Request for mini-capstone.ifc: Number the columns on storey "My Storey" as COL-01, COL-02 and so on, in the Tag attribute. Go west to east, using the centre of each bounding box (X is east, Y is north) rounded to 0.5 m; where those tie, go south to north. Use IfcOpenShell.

First a look at what the model holds.

```python
import ifcopenshell
import ifcopenshell.util.element
import ifcopenshell.util.placement

model = ifcopenshell.open("mini-capstone.ifc")
print(model.schema)
storey = next(s for s in model.by_type("IfcBuildingStorey") if s.Name == "My Storey")
columns = [e for e in ifcopenshell.util.element.get_decomposition(storey) if e.is_a("IfcColumn")]
for e in sorted(columns, key=lambda e: e.id()):
    origin = ifcopenshell.util.placement.get_local_placement(e.ObjectPlacement)[:3, 3]
    print(e.id(), e.Tag, e.Name, origin.round(2) + 0.0, sep=" | ")
```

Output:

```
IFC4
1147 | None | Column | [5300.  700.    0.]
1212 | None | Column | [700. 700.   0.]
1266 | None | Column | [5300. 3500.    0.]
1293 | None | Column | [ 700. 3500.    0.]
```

```python
import ifcopenshell
import ifcopenshell.geom
import ifcopenshell.util.element
import ifcopenshell.util.shape

model = ifcopenshell.open("mini-capstone.ifc")
settings = ifcopenshell.geom.settings()
settings.set("use-world-coords", True)


def centre(element):
    shape = ifcopenshell.geom.create_shape(settings, element)
    return ifcopenshell.util.shape.get_bbox_centroid(shape.geometry)


storey = next(s for s in model.by_type("IfcBuildingStorey") if s.Name == "My Storey")
columns = [e for e in ifcopenshell.util.element.get_decomposition(storey) if e.is_a("IfcColumn")]

# Insertion points can sit at a corner or the storey origin, so sort by the geometry (in metres).
centres = {e: centre(e) for e in columns}
columns.sort(key=lambda e: (round(centres[e][0] / 0.5), centres[e][1]))

for i, e in enumerate(columns, start=1):
    number = f"COL-{i:02d}"
    e.Tag = number
    print(e.id(), number)

model.write("mini-capstone_v2.ifc")
```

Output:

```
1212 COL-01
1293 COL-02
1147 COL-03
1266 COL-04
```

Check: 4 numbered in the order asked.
